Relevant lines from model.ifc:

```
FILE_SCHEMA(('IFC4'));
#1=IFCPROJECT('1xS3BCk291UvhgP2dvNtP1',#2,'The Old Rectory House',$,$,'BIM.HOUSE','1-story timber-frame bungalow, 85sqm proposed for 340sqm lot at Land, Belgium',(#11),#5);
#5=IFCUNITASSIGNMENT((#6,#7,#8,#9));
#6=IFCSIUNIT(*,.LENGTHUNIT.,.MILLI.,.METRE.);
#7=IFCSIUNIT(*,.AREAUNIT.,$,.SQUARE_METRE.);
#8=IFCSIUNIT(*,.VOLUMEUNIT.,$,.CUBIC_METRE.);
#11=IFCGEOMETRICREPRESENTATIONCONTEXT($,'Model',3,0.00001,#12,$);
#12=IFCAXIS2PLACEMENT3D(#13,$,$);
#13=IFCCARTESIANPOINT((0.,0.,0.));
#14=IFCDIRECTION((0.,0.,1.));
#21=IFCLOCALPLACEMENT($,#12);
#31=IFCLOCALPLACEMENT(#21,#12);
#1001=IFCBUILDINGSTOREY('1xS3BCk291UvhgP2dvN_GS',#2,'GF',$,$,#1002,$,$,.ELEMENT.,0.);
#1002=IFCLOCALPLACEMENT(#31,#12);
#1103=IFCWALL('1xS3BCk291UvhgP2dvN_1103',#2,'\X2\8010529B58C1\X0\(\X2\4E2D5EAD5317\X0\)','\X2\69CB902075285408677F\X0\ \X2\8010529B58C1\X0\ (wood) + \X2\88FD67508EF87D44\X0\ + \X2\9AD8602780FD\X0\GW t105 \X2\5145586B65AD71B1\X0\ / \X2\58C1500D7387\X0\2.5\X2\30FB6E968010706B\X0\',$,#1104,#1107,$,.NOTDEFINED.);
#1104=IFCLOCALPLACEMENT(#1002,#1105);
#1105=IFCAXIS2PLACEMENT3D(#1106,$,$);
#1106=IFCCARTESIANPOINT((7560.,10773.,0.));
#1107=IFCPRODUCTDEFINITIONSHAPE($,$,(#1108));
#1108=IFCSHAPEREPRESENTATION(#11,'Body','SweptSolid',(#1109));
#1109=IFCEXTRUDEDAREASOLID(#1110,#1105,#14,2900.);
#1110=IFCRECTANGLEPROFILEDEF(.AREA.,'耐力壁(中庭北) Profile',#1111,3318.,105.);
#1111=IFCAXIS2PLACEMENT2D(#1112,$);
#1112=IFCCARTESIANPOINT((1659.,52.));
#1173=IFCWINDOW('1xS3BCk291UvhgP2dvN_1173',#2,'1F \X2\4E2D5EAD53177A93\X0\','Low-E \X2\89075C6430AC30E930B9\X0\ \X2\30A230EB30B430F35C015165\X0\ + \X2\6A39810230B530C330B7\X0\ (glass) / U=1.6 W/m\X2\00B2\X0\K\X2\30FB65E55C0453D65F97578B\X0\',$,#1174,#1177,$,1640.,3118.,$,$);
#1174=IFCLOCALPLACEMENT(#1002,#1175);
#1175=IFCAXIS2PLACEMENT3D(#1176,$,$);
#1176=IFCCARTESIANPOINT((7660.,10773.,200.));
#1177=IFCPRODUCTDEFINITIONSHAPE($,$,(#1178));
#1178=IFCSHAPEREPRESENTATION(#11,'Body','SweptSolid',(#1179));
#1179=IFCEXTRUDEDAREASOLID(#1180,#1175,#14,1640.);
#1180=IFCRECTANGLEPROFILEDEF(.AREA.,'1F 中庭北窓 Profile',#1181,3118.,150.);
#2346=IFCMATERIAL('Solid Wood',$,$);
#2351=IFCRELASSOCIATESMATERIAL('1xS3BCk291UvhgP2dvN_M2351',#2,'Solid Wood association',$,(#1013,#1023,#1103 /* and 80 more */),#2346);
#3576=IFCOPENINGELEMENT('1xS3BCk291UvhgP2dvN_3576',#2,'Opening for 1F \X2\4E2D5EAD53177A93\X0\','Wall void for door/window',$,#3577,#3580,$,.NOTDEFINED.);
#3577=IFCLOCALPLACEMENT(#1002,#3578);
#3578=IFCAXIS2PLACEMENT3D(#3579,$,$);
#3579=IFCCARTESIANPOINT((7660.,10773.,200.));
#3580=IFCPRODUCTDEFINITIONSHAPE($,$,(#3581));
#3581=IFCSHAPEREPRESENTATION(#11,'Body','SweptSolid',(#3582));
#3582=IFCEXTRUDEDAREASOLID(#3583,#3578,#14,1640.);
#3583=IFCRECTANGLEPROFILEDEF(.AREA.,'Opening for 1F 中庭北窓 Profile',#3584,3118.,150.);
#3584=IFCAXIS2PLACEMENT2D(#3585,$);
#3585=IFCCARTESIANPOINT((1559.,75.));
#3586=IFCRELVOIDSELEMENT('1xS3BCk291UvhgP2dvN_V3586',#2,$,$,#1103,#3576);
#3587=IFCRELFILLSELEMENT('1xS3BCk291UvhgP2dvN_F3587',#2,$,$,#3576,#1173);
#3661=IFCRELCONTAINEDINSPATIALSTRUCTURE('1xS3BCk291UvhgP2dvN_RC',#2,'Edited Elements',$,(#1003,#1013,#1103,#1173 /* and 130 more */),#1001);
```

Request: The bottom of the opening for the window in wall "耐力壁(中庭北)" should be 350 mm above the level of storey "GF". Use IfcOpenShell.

```python
import numpy as np
import ifcopenshell
import ifcopenshell.api.geometry
import ifcopenshell.geom
import ifcopenshell.util.element
import ifcopenshell.util.placement
import ifcopenshell.util.shape
import ifcopenshell.util.unit

model = ifcopenshell.open("model.ifc")
unit_scale = ifcopenshell.util.unit.calculate_unit_scale(model)

window = model.by_guid("1xS3BCk291UvhgP2dvN_1173")
opening = window.FillsVoids[0].RelatingOpeningElement
storey = ifcopenshell.util.element.get_container(window, ifc_class="IfcBuildingStorey")
level = ifcopenshell.util.placement.get_local_placement(storey.ObjectPlacement)[2, 3]

# The opening's origin need not be at the sill, so measure its lowest point.
shape = ifcopenshell.geom.create_shape(ifcopenshell.geom.settings(), opening)
bottom = ifcopenshell.util.shape.get_shape_bottom_elevation(shape, shape.geometry) / unit_scale
dz = level + 350.0 - bottom

shift = np.array([0.0, 0.0, dz])
# The window is not placed relative to its opening, so move both.
for product in (opening, window):
    matrix = ifcopenshell.util.placement.get_local_placement(product.ObjectPlacement)
    matrix[:3, 3] += shift
    ifcopenshell.api.geometry.edit_object_placement(model, product=product, matrix=matrix, is_si=False)

print(f"moved by {dz * unit_scale:+.3f} m")

model.write("model_updated.ifc")
```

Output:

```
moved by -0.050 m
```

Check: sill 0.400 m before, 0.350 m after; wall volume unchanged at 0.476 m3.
